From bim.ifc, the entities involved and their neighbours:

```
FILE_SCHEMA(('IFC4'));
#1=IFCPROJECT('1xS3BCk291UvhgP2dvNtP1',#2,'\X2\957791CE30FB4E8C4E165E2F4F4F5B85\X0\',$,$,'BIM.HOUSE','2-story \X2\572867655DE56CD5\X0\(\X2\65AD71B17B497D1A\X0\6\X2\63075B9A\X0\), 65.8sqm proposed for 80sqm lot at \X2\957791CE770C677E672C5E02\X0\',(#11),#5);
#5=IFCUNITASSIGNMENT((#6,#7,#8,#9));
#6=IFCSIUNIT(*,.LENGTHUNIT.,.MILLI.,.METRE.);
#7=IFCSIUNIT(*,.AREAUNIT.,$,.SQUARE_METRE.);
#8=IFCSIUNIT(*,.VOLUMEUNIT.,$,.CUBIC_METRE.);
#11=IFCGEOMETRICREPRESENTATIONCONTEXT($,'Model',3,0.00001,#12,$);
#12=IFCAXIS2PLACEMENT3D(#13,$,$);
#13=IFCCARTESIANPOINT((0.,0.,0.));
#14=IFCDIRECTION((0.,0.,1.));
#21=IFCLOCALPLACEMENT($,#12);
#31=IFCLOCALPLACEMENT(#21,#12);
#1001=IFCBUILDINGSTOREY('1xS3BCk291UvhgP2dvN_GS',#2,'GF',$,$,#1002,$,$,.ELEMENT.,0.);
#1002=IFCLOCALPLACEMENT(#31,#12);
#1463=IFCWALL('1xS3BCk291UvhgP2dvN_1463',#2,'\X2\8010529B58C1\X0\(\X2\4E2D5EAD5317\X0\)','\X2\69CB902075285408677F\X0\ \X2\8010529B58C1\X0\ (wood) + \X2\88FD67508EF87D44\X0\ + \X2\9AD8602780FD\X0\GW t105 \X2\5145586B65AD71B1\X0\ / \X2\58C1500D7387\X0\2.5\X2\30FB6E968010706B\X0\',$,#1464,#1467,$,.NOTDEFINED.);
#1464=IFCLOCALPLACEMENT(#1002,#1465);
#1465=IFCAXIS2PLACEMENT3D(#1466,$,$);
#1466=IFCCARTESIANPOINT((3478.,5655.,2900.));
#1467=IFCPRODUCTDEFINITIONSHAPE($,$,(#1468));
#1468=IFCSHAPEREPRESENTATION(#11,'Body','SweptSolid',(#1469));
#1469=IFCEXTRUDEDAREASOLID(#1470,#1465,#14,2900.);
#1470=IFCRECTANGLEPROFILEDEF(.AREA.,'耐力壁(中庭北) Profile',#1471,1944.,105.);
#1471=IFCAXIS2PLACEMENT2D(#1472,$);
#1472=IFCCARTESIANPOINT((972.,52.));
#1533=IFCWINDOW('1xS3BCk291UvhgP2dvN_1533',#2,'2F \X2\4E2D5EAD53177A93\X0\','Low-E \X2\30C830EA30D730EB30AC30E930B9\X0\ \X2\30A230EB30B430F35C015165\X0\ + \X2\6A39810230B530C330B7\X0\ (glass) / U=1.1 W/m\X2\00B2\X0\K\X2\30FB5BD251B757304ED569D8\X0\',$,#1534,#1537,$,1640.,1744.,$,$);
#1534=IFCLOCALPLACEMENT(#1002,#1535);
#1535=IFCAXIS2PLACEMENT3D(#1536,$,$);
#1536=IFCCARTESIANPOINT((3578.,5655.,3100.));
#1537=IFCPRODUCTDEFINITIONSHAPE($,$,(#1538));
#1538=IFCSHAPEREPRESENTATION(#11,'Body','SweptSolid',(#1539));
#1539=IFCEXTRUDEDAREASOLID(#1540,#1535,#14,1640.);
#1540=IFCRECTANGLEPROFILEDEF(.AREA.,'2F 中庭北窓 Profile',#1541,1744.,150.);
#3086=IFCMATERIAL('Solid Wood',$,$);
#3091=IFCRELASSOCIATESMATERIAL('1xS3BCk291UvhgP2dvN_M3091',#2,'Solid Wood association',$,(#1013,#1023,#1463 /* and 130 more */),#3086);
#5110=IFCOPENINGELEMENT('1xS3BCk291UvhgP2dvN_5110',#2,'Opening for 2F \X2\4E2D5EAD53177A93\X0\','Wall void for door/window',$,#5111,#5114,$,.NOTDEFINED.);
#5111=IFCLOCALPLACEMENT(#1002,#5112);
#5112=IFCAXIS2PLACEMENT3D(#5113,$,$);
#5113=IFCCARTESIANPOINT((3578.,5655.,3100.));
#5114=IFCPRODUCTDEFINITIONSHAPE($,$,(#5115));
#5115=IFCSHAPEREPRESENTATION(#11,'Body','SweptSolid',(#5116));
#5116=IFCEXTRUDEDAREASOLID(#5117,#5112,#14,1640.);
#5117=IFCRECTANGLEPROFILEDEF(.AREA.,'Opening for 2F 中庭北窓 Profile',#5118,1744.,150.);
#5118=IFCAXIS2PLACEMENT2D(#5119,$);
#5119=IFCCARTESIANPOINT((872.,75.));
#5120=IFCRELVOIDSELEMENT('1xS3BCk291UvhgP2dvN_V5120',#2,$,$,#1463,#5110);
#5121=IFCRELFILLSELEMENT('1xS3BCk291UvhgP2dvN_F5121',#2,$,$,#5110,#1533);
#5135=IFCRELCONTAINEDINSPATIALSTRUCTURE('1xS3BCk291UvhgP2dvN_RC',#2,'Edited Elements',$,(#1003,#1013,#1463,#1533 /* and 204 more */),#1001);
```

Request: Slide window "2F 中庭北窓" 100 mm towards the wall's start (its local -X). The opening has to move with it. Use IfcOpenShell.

```python
import ifcopenshell
import ifcopenshell.api.geometry
import ifcopenshell.util.placement

model = ifcopenshell.open("bim.ifc")

window = model.by_id(1533)
opening = window.FillsVoids[0].RelatingOpeningElement
wall = opening.VoidsElements[0].RelatingBuildingElement

wall_matrix = ifcopenshell.util.placement.get_local_placement(wall.ObjectPlacement)
shift = wall_matrix[:3, 0] * -100.0
before = ifcopenshell.util.placement.get_local_placement(window.ObjectPlacement)[:3, 3].copy()

# The window is not placed relative to its opening, so move both.
for product in (opening, window):
    matrix = ifcopenshell.util.placement.get_local_placement(product.ObjectPlacement)
    matrix[:3, 3] += shift
    ifcopenshell.api.geometry.edit_object_placement(model, product=product, matrix=matrix, is_si=False)

after = ifcopenshell.util.placement.get_local_placement(window.ObjectPlacement)[:3, 3]
print("window moved by", (after - before).round(3) + 0.0)

model.write("bim_edited.ifc")
```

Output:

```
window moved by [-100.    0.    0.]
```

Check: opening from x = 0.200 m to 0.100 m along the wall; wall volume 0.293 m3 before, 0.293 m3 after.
